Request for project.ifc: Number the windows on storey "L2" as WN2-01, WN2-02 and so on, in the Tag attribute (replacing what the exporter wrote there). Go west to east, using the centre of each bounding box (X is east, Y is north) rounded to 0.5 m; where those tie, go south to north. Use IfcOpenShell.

First a look at what the model holds.

```python
import ifcopenshell
import ifcopenshell.util.element
import ifcopenshell.util.placement

model = ifcopenshell.open("project.ifc")
print(model.schema)
storey = next(s for s in model.by_type("IfcBuildingStorey") if s.Name == "L2")
windows = [e for e in ifcopenshell.util.element.get_decomposition(storey) if e.is_a("IfcWindow")]
for e in sorted(windows, key=lambda e: e.id()):
    origin = ifcopenshell.util.placement.get_local_placement(e.ObjectPlacement)[:3, 3]
    print(e.id(), e.Tag, e.Name, origin.round(2) + 0.0, sep=" | ")
```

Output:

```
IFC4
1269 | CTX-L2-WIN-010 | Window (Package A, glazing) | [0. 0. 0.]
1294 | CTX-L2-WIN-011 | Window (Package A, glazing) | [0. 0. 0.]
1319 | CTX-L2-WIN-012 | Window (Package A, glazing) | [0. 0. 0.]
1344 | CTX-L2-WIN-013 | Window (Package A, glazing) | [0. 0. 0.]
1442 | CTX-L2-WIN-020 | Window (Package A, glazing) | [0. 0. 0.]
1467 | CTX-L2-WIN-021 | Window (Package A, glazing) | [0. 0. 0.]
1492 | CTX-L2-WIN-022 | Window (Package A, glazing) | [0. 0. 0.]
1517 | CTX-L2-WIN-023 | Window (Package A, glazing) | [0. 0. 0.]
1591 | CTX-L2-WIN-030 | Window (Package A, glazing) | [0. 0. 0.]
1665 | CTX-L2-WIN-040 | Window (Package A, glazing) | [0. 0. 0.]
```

```python
import ifcopenshell
import ifcopenshell.geom
import ifcopenshell.util.element
import ifcopenshell.util.shape

model = ifcopenshell.open("project.ifc")
settings = ifcopenshell.geom.settings()
settings.set("use-world-coords", True)


def centre(element):
    shape = ifcopenshell.geom.create_shape(settings, element)
    return ifcopenshell.util.shape.get_bbox_centroid(shape.geometry)


storey = next(s for s in model.by_type("IfcBuildingStorey") if s.Name == "L2")
windows = [e for e in ifcopenshell.util.element.get_decomposition(storey) if e.is_a("IfcWindow")]

# Insertion points can sit at a corner or the storey origin, so sort by the geometry (in metres).
centres = {e: centre(e) for e in windows}
windows.sort(key=lambda e: (round(centres[e][0] / 0.5), centres[e][1]))

for i, e in enumerate(windows, start=1):
    number = f"WN2-{i:02d}"
    e.Tag = number
    print(e.id(), number)

model.write("project_updated.ifc")
```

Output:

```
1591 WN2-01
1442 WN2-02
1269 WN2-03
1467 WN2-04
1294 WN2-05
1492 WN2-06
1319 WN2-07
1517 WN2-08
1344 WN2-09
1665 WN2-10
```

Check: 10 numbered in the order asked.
